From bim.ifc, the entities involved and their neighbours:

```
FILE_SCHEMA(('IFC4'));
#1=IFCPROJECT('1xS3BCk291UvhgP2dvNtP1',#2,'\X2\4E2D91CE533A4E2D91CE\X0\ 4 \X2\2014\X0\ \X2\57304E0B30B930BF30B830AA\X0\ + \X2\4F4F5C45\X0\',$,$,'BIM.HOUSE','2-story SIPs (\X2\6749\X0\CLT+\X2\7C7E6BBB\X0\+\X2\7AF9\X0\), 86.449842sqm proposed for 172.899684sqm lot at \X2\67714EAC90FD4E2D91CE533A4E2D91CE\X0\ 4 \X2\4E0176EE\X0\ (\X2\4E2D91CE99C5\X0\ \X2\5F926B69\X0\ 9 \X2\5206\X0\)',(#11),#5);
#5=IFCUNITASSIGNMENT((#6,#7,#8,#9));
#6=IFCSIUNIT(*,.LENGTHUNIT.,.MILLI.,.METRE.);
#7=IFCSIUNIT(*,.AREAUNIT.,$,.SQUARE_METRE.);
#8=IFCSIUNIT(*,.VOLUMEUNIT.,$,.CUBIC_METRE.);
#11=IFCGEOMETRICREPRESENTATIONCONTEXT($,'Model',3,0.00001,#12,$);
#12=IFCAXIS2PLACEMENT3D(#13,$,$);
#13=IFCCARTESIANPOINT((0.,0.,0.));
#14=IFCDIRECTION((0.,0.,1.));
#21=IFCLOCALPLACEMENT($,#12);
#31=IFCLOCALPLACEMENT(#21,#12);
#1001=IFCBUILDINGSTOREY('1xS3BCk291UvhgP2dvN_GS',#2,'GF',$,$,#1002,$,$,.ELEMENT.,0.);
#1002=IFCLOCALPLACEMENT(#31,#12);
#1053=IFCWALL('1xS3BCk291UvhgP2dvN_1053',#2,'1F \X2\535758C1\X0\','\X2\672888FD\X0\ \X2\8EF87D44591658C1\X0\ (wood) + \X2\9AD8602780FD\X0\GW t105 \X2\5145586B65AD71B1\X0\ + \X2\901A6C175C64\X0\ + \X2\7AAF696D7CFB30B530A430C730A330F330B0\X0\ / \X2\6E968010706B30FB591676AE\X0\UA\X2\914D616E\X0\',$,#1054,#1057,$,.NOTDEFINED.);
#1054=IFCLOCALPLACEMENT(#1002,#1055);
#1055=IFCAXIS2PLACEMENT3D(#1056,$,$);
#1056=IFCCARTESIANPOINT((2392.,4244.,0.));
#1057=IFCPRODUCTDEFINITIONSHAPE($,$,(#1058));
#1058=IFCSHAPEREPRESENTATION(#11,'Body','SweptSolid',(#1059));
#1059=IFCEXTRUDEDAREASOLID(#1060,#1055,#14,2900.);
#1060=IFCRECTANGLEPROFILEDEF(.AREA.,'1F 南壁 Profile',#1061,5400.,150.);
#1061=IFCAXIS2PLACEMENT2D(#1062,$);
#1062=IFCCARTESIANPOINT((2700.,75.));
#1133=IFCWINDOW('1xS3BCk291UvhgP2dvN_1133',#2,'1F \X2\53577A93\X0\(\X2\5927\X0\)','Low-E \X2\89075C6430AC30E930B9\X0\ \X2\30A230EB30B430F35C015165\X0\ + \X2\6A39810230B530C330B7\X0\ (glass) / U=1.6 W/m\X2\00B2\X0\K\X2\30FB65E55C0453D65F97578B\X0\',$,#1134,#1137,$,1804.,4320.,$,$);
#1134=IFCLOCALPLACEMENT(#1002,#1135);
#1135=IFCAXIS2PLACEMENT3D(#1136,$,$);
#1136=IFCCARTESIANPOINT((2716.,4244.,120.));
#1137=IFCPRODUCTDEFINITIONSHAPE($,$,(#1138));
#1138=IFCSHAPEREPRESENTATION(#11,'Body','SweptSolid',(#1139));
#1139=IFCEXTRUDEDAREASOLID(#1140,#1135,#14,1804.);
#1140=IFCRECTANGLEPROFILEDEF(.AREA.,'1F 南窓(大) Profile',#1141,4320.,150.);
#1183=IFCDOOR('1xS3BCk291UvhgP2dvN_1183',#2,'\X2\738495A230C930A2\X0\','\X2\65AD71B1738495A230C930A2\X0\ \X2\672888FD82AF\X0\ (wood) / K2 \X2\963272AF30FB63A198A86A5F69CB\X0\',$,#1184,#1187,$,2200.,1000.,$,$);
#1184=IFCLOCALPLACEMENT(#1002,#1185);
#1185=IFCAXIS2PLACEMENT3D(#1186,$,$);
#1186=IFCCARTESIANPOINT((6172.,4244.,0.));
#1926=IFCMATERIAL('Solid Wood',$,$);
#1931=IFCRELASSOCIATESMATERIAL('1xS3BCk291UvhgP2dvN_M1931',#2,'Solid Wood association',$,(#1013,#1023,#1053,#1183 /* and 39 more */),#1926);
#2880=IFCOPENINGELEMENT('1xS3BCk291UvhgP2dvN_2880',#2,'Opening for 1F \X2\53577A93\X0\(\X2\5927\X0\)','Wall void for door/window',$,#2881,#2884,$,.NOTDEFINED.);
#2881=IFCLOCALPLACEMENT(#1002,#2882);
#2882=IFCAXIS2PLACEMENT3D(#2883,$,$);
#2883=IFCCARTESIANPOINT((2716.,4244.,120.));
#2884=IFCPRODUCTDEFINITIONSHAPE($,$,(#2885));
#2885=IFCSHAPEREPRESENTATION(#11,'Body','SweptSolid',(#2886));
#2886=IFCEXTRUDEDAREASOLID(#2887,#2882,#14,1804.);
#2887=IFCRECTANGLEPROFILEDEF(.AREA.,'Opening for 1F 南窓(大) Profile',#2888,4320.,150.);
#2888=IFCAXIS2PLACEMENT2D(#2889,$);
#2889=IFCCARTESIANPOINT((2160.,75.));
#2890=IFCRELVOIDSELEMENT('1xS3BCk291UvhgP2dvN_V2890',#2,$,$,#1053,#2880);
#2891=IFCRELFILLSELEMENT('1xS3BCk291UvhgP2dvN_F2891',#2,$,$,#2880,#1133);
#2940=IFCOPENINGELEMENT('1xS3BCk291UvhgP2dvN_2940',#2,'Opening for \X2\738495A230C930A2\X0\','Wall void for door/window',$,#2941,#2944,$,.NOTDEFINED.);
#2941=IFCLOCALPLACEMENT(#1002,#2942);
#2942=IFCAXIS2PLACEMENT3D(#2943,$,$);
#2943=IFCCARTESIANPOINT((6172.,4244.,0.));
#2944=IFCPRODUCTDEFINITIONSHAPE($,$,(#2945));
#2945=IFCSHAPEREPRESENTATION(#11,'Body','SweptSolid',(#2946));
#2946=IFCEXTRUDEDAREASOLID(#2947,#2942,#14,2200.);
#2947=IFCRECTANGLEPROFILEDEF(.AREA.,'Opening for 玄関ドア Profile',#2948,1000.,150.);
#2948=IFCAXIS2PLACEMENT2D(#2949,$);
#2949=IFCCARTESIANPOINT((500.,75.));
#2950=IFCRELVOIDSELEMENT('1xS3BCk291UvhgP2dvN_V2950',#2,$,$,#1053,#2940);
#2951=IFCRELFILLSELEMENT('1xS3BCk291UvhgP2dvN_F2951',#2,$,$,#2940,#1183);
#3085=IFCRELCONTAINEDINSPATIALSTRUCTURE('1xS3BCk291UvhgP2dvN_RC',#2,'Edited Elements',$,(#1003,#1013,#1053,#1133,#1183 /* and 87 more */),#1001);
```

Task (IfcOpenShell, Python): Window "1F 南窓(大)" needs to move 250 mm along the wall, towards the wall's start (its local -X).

```python
import ifcopenshell
import ifcopenshell.api.geometry
import ifcopenshell.util.placement
import ifcopenshell.util.unit

model = ifcopenshell.open("bim.ifc")
unit_scale = ifcopenshell.util.unit.calculate_unit_scale(model)

window = model.by_guid("1xS3BCk291UvhgP2dvN_1133")
opening = window.FillsVoids[0].RelatingOpeningElement
wall = opening.VoidsElements[0].RelatingBuildingElement

wall_matrix = ifcopenshell.util.placement.get_local_placement(wall.ObjectPlacement)
shift = wall_matrix[:3, 0] * -0.25 / unit_scale
before = ifcopenshell.util.placement.get_local_placement(window.ObjectPlacement)[:3, 3].copy()

# The window is not placed relative to its opening, so move both.
for product in (opening, window):
    matrix = ifcopenshell.util.placement.get_local_placement(product.ObjectPlacement)
    matrix[:3, 3] += shift
    ifcopenshell.api.geometry.edit_object_placement(model, product=product, matrix=matrix, is_si=False)

after = ifcopenshell.util.placement.get_local_placement(window.ObjectPlacement)[:3, 3]
print("window moved by", (after - before).round(3) + 0.0)

model.write("bim_updated.ifc")
```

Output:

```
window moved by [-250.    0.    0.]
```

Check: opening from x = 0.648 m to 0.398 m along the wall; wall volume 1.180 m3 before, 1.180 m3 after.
